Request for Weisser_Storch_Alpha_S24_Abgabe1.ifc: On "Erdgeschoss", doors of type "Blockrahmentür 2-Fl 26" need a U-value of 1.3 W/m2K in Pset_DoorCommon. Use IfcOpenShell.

First a look at what the model holds.

```python
import ifcopenshell
import ifcopenshell.util.element

model = ifcopenshell.open("Weisser_Storch_Alpha_S24_Abgabe1.ifc")
print(model.schema)
storey = next(s for s in model.by_type("IfcBuildingStorey") if s.Name == "Erdgeschoss")
doors = [e for e in ifcopenshell.util.element.get_decomposition(storey) if e.is_a("IfcDoor")]
seen = {}
for e in doors:
    element_type = ifcopenshell.util.element.get_type(e)
    key = (element_type.Name if element_type != e and element_type else None, ifcopenshell.util.element.get_pset(e, "Pset_DoorCommon", "ThermalTransmittance"))
    seen[key] = seen.get(key, 0) + 1
for (name, value), count in sorted(seen.items(), key=str):
    print(count, "x", name, "|", value)
```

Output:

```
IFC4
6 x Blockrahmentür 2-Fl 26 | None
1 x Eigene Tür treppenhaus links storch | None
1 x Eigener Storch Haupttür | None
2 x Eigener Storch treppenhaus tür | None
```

```python
import ifcopenshell
import ifcopenshell.api.pset
import ifcopenshell.util.element

model = ifcopenshell.open("Weisser_Storch_Alpha_S24_Abgabe1.ifc")

storey = next(s for s in model.by_type("IfcBuildingStorey") if s.Name == "Erdgeschoss")
doors = [e for e in ifcopenshell.util.element.get_decomposition(storey) if e.is_a("IfcDoor")]

count = 0
for e in doors:
    element_type = ifcopenshell.util.element.get_type(e)
    if element_type in (None, e) or element_type.Name != "Blockrahmentür 2-Fl 26":
        continue
    # add_pset returns the element's existing set when there is one.
    pset = ifcopenshell.api.pset.add_pset(model, product=e, name="Pset_DoorCommon")
    ifcopenshell.api.pset.edit_pset(model, pset=pset, properties={"ThermalTransmittance": 1.3})
    count += 1

print(count, "doors updated")

model.write("Weisser_Storch_Alpha_S24_Abgabe1_v2.ifc")
```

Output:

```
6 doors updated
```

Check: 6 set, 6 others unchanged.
